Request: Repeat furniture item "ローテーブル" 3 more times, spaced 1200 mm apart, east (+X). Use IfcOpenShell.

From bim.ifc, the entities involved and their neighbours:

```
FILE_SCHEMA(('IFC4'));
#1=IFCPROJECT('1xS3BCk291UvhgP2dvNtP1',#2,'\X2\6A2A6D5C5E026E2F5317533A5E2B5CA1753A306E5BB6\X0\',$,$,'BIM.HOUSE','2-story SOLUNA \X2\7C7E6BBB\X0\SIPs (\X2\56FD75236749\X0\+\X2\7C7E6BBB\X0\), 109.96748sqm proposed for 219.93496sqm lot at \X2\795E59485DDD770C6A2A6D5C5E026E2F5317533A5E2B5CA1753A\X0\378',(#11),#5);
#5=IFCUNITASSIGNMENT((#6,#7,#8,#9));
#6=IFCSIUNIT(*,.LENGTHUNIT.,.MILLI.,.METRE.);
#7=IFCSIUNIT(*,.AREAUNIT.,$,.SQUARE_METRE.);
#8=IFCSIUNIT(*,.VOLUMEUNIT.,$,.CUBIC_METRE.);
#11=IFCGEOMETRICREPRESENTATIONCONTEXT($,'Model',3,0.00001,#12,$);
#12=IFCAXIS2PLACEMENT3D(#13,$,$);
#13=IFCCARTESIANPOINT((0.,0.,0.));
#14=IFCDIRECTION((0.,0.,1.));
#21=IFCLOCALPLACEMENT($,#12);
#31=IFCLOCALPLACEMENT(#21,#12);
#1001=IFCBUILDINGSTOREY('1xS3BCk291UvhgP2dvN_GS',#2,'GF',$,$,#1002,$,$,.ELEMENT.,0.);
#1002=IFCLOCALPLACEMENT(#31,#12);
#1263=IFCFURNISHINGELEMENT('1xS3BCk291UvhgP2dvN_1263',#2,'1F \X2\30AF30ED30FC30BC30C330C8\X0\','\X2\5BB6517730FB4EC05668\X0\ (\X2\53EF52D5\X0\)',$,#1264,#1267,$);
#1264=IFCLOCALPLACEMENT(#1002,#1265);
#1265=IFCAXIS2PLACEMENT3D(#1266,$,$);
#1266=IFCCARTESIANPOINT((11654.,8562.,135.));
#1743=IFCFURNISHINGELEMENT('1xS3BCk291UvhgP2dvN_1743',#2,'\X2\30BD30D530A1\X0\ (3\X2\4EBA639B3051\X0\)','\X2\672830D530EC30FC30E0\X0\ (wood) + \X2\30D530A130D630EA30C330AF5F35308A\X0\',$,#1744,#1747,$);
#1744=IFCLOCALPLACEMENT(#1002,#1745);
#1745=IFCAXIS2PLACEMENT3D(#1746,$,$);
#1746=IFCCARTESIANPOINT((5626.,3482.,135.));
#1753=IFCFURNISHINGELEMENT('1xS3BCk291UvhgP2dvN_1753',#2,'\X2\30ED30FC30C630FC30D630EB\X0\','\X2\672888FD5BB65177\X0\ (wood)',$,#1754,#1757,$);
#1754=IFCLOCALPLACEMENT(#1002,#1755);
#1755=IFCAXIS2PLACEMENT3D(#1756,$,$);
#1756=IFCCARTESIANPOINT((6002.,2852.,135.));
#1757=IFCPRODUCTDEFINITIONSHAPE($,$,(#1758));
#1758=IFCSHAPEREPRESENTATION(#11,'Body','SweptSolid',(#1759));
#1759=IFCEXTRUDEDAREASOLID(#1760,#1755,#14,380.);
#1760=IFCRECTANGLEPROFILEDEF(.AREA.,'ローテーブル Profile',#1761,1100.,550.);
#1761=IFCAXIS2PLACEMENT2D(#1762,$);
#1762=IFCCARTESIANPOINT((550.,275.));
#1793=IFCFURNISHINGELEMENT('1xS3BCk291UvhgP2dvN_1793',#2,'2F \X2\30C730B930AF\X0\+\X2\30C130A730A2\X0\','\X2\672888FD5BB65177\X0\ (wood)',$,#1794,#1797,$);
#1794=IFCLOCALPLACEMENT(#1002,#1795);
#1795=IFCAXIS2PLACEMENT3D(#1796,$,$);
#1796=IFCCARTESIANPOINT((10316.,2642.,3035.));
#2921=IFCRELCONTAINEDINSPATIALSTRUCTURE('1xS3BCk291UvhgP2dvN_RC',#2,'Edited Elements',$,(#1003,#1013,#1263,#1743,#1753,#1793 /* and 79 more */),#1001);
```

```python
import numpy as np
import ifcopenshell
import ifcopenshell.api.geometry
import ifcopenshell.api.root
import ifcopenshell.util.element
import ifcopenshell.util.placement

model = ifcopenshell.open("bim.ifc")


def reuse_history(source, copy):
    """copy_class also copies each property set's owner history, people and application; keep the originals."""
    for rel in copy.IsDefinedBy:
        if rel.is_a("IfcRelDefinesByProperties") and (history := rel.RelatingPropertyDefinition.OwnerHistory):
            rel.RelatingPropertyDefinition.OwnerHistory = source.OwnerHistory
            ifcopenshell.util.element.remove_deep2(model, history)


source = model.by_id(1753)
base = ifcopenshell.util.placement.get_local_placement(source.ObjectPlacement)
step = np.array([1.0, 0.0, 0.0]) * 1200.0

for i in range(1, 4):
    copy = ifcopenshell.api.root.copy_class(model, product=source)
    copy.Representation = ifcopenshell.util.element.copy_deep(
        model, source.Representation, exclude=["IfcGeometricRepresentationContext", "IfcRepresentationMap"]
    )
    reuse_history(source, copy)
    matrix = base.copy()
    matrix[:3, 3] += i * step
    print("added at", matrix[:3, 3].round(3) + 0.0)
    ifcopenshell.api.geometry.edit_object_placement(model, product=copy, matrix=matrix, is_si=False)

model.write("bim_updated.ifc")
```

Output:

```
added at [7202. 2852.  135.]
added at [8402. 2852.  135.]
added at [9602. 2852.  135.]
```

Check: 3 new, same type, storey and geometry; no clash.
